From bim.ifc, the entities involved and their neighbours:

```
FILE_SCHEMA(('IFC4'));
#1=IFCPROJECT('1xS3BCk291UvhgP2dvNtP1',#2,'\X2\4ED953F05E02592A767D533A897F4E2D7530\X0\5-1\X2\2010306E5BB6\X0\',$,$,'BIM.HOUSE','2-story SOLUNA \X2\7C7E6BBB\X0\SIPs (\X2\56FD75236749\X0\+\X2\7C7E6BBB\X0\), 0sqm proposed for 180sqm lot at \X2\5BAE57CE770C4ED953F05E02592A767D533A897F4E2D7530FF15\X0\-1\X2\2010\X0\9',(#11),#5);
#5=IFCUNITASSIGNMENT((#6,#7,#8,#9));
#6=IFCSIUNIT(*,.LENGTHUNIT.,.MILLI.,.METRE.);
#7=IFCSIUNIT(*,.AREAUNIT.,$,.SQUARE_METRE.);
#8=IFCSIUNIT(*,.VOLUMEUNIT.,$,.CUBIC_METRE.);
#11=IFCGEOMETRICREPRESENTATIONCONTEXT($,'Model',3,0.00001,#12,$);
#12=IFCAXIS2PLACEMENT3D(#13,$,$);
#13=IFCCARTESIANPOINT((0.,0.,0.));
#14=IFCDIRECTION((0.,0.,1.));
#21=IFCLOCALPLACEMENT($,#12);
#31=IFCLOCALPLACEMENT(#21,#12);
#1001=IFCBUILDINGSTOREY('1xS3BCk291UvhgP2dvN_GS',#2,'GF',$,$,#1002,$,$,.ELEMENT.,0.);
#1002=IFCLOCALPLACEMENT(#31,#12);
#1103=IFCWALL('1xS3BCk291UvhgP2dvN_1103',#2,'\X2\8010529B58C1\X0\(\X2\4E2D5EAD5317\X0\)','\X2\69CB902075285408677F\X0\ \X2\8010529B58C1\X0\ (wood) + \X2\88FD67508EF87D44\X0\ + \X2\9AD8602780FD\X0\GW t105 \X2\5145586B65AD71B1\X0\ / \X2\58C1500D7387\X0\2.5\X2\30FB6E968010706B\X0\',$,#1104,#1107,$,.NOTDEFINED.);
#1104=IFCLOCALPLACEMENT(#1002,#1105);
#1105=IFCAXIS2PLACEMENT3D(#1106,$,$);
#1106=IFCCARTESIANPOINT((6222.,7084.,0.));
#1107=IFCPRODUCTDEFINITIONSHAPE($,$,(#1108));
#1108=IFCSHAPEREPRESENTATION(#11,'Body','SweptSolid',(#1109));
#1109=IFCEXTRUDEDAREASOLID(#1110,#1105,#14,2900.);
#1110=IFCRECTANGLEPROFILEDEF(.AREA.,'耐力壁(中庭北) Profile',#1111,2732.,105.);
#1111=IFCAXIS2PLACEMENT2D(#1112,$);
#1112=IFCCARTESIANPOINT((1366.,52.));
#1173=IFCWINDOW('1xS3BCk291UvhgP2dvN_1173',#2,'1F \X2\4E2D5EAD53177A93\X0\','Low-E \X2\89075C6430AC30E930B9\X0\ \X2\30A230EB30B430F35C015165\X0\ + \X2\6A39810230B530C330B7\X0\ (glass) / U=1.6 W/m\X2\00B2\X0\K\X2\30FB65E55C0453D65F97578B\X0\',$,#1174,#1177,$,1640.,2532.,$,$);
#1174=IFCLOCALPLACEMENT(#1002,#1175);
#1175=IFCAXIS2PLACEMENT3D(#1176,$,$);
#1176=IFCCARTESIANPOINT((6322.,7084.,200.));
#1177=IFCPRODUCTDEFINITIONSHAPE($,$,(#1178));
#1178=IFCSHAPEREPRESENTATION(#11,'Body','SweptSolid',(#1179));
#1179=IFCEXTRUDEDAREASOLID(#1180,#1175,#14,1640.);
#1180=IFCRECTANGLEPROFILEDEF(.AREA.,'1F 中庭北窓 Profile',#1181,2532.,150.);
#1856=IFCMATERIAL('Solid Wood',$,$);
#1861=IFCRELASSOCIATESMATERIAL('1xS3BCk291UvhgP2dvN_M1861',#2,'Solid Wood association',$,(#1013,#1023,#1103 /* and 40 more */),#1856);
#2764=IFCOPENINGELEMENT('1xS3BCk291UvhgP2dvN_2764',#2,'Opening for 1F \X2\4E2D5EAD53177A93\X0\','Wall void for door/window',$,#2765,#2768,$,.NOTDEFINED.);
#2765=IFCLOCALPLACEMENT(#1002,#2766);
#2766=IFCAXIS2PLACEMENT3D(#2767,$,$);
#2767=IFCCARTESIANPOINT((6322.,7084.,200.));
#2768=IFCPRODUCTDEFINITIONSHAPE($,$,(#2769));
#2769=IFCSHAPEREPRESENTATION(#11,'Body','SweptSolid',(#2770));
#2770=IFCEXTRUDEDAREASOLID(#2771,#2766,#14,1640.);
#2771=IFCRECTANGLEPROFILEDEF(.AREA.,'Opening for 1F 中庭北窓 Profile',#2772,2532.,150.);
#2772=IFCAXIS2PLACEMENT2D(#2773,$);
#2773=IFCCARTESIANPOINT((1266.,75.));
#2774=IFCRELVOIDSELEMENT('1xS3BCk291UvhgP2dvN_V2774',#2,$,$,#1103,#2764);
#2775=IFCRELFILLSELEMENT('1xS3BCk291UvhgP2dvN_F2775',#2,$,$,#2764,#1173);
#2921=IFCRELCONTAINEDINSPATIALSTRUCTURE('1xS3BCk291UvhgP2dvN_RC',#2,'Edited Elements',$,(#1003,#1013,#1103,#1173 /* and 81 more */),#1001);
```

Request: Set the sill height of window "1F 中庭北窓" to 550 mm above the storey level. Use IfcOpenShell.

```python
import numpy as np
import ifcopenshell
import ifcopenshell.api.geometry
import ifcopenshell.geom
import ifcopenshell.util.element
import ifcopenshell.util.placement
import ifcopenshell.util.shape
import ifcopenshell.util.unit

model = ifcopenshell.open("bim.ifc")
unit_scale = ifcopenshell.util.unit.calculate_unit_scale(model)

window = model.by_guid("1xS3BCk291UvhgP2dvN_1173")
opening = window.FillsVoids[0].RelatingOpeningElement
storey = ifcopenshell.util.element.get_container(window, ifc_class="IfcBuildingStorey")
level = ifcopenshell.util.placement.get_local_placement(storey.ObjectPlacement)[2, 3]

# The opening's origin need not be at the sill, so measure its lowest point.
shape = ifcopenshell.geom.create_shape(ifcopenshell.geom.settings(), opening)
bottom = ifcopenshell.util.shape.get_shape_bottom_elevation(shape, shape.geometry) / unit_scale
dz = level + 0.55 / unit_scale - bottom

shift = np.array([0.0, 0.0, dz])
# The window is not placed relative to its opening, so move both.
for product in (opening, window):
    matrix = ifcopenshell.util.placement.get_local_placement(product.ObjectPlacement)
    matrix[:3, 3] += shift
    ifcopenshell.api.geometry.edit_object_placement(model, product=product, matrix=matrix, is_si=False)

print(f"moved by {dz * unit_scale:+.3f} m")

model.write("bim_updated.ifc")
```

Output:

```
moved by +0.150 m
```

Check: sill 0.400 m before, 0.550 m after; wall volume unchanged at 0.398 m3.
